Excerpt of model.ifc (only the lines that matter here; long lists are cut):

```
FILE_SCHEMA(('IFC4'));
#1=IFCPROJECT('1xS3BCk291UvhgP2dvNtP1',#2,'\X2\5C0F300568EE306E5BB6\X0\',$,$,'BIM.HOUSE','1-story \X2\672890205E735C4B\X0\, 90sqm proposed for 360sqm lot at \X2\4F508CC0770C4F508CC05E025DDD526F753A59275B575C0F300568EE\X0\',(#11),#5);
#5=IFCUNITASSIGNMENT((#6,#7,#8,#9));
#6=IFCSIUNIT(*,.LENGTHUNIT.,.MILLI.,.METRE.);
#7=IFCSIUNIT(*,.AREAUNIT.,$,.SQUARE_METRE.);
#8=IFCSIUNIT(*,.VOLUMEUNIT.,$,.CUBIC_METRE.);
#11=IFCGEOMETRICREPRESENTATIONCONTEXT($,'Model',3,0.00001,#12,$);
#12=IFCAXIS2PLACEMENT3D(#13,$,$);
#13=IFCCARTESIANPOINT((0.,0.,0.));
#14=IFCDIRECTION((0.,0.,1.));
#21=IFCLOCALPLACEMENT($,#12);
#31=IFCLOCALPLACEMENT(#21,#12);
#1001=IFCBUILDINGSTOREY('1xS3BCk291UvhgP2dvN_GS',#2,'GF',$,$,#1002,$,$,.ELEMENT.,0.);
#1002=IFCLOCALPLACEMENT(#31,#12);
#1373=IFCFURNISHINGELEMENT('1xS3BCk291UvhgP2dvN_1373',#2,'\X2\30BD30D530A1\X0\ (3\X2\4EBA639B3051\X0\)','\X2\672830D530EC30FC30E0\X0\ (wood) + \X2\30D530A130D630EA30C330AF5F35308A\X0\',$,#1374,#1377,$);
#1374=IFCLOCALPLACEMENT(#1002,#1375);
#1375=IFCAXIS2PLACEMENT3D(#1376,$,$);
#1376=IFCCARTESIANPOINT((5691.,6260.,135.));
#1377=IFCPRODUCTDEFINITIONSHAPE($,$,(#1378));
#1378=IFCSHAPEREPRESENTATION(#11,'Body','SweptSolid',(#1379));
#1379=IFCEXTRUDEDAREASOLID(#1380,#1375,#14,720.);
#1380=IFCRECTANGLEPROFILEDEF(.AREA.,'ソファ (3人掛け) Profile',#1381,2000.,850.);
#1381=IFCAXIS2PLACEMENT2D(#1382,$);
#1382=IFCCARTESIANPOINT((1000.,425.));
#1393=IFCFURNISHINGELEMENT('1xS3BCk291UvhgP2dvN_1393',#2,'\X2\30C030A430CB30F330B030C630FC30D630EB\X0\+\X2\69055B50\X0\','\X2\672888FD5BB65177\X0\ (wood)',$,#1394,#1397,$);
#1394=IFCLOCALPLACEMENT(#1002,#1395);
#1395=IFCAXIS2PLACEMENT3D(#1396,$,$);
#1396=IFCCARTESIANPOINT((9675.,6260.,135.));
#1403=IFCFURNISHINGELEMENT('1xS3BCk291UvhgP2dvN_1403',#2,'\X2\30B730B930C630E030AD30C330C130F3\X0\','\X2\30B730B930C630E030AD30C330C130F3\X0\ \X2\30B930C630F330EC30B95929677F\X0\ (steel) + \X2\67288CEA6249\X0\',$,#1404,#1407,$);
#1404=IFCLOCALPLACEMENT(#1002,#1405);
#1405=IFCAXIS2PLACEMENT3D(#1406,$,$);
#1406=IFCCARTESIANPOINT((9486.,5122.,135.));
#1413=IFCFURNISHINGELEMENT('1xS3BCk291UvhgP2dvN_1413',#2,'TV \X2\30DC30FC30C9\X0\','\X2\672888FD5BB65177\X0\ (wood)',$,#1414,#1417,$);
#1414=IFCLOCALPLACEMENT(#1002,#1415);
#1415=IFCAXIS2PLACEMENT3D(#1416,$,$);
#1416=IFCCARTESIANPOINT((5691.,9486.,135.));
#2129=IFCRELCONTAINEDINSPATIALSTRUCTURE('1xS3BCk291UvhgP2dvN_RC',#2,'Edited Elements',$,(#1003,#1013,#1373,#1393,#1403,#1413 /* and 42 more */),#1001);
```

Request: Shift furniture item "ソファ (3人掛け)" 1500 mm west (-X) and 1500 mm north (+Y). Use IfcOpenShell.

```python
import ifcopenshell
import ifcopenshell.api.geometry
import ifcopenshell.util.placement

model = ifcopenshell.open("model.ifc")

item = model.by_guid("1xS3BCk291UvhgP2dvN_1373")
matrix = ifcopenshell.util.placement.get_local_placement(item.ObjectPlacement)
matrix[0, 3] -= 1500.0
matrix[1, 3] += 1500.0
ifcopenshell.api.geometry.edit_object_placement(model, product=item, matrix=matrix, is_si=False)

print(ifcopenshell.util.placement.get_local_placement(item.ObjectPlacement).round(3) + 0.0)

model.write("model_v2.ifc")
```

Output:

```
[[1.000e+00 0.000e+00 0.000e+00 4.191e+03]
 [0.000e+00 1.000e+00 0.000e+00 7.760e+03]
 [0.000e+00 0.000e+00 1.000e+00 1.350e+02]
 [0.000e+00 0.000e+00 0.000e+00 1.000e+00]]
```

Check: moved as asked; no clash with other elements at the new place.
